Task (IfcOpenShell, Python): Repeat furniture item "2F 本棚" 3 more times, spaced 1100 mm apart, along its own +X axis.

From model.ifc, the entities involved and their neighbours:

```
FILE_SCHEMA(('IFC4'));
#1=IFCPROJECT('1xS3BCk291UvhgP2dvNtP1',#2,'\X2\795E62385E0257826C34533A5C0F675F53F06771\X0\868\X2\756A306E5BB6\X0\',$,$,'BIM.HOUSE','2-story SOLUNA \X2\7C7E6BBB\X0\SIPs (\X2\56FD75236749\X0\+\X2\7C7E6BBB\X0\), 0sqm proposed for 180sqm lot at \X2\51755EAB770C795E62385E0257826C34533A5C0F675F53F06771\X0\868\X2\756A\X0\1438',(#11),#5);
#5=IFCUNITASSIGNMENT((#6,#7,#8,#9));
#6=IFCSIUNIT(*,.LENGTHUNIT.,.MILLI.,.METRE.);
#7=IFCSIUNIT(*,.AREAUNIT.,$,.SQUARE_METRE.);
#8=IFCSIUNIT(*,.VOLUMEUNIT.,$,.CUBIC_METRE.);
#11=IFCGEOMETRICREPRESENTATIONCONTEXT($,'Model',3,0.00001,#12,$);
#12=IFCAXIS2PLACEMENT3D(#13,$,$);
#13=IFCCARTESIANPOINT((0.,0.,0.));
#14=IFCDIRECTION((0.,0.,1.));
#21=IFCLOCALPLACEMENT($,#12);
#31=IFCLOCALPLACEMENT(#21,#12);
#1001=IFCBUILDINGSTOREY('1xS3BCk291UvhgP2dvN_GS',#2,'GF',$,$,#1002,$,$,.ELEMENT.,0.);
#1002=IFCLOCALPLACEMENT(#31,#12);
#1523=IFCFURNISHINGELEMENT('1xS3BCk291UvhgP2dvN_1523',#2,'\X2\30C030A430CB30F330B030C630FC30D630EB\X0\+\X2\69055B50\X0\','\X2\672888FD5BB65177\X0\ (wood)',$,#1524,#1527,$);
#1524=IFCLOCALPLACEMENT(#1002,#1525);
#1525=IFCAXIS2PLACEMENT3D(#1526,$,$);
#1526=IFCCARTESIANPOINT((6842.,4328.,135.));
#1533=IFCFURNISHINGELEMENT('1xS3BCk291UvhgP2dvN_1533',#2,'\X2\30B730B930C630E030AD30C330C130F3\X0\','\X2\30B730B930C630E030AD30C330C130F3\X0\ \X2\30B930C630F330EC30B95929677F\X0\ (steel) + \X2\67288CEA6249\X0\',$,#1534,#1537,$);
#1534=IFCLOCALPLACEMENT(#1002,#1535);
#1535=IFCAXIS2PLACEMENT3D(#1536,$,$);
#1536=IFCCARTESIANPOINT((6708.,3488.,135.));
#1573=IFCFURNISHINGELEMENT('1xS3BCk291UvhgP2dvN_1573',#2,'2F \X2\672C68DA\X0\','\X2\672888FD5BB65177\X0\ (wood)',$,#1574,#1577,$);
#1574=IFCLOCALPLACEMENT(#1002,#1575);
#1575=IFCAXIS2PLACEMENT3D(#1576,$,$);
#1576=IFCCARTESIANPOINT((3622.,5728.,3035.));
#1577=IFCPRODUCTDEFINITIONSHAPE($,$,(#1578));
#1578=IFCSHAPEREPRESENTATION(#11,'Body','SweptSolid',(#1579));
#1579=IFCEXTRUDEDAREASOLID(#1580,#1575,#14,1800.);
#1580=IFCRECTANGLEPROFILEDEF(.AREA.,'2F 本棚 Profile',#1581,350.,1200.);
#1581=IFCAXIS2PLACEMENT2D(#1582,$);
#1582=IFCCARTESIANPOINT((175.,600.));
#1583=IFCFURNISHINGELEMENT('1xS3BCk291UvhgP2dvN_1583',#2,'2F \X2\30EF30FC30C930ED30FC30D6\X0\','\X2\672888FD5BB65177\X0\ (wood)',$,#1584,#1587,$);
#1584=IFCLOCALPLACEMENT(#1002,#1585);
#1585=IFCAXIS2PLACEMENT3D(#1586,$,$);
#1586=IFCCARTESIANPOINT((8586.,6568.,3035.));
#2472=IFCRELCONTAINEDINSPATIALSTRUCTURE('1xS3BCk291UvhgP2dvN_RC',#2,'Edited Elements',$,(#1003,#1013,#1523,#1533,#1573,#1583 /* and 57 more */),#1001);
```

```python
import ifcopenshell
import ifcopenshell.api.geometry
import ifcopenshell.api.root
import ifcopenshell.util.element
import ifcopenshell.util.placement
import ifcopenshell.util.unit

model = ifcopenshell.open("model.ifc")
unit_scale = ifcopenshell.util.unit.calculate_unit_scale(model)


def reuse_history(source, copy):
    """copy_class also copies each property set's owner history, people and application; keep the originals."""
    for rel in copy.IsDefinedBy:
        if rel.is_a("IfcRelDefinesByProperties") and (history := rel.RelatingPropertyDefinition.OwnerHistory):
            rel.RelatingPropertyDefinition.OwnerHistory = source.OwnerHistory
            ifcopenshell.util.element.remove_deep2(model, history)


source = model.by_id(1573)
base = ifcopenshell.util.placement.get_local_placement(source.ObjectPlacement)
step = base[:3, 0] * 1.1 / unit_scale

for i in range(1, 4):
    copy = ifcopenshell.api.root.copy_class(model, product=source)
    copy.Representation = ifcopenshell.util.element.copy_deep(
        model, source.Representation, exclude=["IfcGeometricRepresentationContext", "IfcRepresentationMap"]
    )
    reuse_history(source, copy)
    matrix = base.copy()
    matrix[:3, 3] += i * step
    print("added at", matrix[:3, 3].round(3) + 0.0)
    ifcopenshell.api.geometry.edit_object_placement(model, product=copy, matrix=matrix, is_si=False)

model.write("model_v2.ifc")
```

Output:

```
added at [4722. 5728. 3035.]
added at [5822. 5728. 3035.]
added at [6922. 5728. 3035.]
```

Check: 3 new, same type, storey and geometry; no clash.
